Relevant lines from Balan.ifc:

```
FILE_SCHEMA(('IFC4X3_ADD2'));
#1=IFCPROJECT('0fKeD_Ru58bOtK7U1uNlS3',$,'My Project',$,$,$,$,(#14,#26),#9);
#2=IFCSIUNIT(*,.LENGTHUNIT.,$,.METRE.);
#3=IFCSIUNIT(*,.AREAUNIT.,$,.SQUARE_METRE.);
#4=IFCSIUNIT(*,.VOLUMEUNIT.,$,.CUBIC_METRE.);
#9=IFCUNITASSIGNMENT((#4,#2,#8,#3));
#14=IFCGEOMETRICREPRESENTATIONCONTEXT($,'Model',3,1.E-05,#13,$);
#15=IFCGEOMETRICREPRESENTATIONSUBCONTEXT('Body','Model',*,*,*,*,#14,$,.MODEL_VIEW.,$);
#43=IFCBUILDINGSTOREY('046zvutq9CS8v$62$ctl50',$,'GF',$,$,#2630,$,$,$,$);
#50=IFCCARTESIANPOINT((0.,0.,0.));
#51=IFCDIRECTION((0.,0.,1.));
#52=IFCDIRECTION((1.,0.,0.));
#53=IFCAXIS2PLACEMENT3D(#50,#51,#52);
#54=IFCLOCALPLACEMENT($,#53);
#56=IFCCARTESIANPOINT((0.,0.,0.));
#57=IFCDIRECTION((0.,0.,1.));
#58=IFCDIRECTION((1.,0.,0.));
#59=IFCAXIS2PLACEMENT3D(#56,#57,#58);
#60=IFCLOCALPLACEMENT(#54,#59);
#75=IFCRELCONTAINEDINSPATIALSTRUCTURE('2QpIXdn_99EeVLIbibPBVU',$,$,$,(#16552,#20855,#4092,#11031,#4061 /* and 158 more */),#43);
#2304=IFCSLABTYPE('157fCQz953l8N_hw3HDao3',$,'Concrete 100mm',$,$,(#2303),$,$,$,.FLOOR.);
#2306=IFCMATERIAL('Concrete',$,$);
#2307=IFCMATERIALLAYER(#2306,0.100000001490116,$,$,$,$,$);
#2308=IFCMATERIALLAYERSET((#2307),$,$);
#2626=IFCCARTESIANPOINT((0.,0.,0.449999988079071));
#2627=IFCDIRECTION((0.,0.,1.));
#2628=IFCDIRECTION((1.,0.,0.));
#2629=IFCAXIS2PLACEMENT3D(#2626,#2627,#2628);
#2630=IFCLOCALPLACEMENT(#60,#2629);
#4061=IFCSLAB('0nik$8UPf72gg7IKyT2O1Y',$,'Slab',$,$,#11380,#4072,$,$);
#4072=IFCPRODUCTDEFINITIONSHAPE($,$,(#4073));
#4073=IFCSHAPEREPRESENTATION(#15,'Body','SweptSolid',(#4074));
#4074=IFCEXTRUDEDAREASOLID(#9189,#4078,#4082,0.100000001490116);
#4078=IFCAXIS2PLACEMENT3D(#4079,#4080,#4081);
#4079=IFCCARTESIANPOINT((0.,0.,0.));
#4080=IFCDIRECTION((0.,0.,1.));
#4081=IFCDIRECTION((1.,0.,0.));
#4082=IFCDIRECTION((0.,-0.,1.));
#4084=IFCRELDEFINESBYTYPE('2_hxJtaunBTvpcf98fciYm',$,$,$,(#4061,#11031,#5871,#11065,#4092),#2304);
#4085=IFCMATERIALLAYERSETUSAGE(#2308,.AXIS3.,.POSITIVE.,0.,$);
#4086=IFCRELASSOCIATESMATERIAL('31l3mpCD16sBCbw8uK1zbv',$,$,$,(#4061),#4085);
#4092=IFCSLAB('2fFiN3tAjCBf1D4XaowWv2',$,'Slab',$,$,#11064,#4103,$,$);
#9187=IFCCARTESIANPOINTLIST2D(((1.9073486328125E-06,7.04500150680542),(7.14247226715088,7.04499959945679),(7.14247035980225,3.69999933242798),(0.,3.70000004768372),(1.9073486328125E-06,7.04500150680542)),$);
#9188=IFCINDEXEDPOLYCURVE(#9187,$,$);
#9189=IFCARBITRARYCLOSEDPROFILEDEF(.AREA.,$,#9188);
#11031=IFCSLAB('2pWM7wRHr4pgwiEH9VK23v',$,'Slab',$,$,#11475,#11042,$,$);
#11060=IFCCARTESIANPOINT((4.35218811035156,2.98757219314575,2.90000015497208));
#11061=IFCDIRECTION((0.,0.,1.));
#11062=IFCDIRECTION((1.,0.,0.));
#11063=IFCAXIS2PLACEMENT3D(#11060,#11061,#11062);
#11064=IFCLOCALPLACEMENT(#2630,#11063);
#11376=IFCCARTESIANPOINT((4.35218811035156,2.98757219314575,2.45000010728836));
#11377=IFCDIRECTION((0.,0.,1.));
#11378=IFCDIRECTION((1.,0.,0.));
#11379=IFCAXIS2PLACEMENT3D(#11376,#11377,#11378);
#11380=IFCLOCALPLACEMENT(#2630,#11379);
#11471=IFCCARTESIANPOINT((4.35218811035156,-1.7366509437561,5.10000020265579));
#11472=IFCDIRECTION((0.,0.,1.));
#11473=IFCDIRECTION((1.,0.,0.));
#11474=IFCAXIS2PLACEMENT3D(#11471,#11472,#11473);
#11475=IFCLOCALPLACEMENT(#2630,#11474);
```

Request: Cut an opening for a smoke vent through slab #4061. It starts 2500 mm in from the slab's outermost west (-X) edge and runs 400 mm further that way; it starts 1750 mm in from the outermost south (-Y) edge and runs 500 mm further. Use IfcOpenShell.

```python
import numpy as np
import ifcopenshell
import ifcopenshell.api.feature
import ifcopenshell.api.geometry
import ifcopenshell.api.root
import ifcopenshell.geom
import ifcopenshell.util.placement
import ifcopenshell.util.representation
import ifcopenshell.util.shape
import ifcopenshell.util.unit

model = ifcopenshell.open("Balan.ifc")
unit_scale = ifcopenshell.util.unit.calculate_unit_scale(model)
settings = ifcopenshell.geom.settings()


def volume(element):
    """Net volume in cubic metres, openings subtracted."""
    shape = ifcopenshell.geom.create_shape(settings, element)
    return ifcopenshell.util.shape.get_volume(shape.geometry)


slab = model.by_guid("0nik$8UPf72gg7IKyT2O1Y")
before = volume(slab)

# Extent in the slab's own axes, in metres. The edges named are its -X and -Y sides.
slab_shape = ifcopenshell.geom.create_shape(settings, slab)
vertices = ifcopenshell.util.shape.get_vertices(slab_shape.geometry)
x_min, y_min, bottom = vertices.min(axis=0)
top = vertices[:, 2].max()

opening = ifcopenshell.api.root.create_entity(model, ifc_class="IfcOpeningElement", name="Smoke vent opening", predefined_type="OPENING")
context = ifcopenshell.util.representation.get_context(model, "Model", "Body", "MODEL_VIEW")
width, depth = 0.4, 0.5
outline = [(0.0, 0.0), (width, 0.0), (width, depth), (0.0, depth), (0.0, 0.0)]
# Overshoot both faces by 50 mm so the cut is clean.
shape = ifcopenshell.api.geometry.add_slab_representation(
    model, context=context, depth=top - bottom + 0.1, polyline=outline
)
ifcopenshell.api.geometry.assign_representation(model, product=opening, representation=shape)

matrix = ifcopenshell.util.placement.get_local_placement(slab.ObjectPlacement)
matrix[:, 3] = matrix @ np.append(np.array([x_min + 2.5, y_min + 1.75, bottom - 0.05]) / unit_scale, 1.0)
ifcopenshell.api.geometry.edit_object_placement(model, product=opening, matrix=matrix, is_si=False)
ifcopenshell.api.feature.add_feature(model, feature=opening, element=slab)

after = volume(slab)

print(f"slab volume {before:.3f} -> {after:.3f} m3")

model.write("Balan_edited.ifc")
```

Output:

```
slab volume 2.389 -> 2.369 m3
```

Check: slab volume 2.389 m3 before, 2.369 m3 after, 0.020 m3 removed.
